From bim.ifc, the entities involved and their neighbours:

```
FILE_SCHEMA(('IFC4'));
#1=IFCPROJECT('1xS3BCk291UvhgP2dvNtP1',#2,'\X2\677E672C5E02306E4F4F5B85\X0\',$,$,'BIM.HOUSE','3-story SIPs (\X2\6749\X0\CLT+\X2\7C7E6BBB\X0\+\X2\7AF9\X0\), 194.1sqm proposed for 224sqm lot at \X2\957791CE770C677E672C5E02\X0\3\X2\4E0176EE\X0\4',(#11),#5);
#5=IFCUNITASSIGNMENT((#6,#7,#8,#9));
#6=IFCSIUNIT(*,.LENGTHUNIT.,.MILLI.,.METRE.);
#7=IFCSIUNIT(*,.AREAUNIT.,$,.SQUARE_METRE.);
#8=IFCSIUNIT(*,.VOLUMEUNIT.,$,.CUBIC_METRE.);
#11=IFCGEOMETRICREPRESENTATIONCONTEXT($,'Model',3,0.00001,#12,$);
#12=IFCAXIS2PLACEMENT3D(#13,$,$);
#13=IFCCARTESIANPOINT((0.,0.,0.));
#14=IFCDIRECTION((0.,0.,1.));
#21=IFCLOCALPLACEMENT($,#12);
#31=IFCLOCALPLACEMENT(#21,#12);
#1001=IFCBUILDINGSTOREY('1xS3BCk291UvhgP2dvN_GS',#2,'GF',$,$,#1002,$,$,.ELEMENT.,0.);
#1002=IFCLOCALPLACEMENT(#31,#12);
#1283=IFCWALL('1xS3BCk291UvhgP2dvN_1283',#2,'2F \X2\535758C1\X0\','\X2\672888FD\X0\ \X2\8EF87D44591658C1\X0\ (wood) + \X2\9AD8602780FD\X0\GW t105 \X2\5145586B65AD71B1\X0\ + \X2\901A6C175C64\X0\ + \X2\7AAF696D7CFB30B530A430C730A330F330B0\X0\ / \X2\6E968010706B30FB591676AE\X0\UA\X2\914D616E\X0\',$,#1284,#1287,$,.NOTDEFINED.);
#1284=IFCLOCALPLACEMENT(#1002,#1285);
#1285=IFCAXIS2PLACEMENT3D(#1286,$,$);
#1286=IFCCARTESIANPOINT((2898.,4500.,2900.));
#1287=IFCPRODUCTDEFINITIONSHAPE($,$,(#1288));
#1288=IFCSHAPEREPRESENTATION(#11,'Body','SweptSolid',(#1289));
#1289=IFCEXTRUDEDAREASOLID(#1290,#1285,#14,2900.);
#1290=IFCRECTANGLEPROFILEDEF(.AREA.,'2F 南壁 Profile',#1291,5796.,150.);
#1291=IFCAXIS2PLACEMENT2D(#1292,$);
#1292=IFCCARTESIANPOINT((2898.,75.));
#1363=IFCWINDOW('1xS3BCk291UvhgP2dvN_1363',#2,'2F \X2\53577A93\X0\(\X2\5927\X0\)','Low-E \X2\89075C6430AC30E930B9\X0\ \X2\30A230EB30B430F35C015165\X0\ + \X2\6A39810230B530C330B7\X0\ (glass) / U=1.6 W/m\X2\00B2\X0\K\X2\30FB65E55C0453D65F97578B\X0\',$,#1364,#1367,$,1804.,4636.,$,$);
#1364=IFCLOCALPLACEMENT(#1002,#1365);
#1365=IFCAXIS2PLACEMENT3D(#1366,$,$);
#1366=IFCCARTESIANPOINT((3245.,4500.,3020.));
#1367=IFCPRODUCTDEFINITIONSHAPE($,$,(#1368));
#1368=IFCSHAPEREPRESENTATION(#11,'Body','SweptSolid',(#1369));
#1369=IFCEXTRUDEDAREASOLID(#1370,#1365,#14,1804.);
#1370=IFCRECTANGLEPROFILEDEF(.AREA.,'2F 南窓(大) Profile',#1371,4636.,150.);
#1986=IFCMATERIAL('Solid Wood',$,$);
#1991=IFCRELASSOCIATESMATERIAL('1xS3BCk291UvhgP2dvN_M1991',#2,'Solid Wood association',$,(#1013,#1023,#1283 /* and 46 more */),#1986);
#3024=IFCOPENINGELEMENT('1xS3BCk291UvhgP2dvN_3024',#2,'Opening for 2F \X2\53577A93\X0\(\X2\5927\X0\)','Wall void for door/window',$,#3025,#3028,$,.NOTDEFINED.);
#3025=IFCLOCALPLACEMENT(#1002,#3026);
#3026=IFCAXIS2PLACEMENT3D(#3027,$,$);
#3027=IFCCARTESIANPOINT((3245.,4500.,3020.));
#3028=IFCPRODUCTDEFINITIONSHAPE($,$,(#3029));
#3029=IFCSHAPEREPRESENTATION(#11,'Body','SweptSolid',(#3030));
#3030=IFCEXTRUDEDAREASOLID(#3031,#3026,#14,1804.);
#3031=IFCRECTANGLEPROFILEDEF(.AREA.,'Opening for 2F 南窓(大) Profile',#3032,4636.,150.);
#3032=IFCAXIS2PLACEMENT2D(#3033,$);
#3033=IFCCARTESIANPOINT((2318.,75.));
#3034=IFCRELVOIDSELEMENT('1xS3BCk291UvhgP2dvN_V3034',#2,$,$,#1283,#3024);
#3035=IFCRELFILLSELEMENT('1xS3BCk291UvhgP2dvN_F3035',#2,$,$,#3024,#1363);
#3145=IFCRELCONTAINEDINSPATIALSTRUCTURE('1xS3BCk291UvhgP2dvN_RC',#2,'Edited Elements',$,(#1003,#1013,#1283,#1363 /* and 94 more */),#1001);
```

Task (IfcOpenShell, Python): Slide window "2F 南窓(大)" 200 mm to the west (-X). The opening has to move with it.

```python
import ifcopenshell
import ifcopenshell.api.geometry
import ifcopenshell.util.placement

model = ifcopenshell.open("bim.ifc")

window = model.by_guid("1xS3BCk291UvhgP2dvN_1363")
opening = window.FillsVoids[0].RelatingOpeningElement
wall = opening.VoidsElements[0].RelatingBuildingElement

wall_matrix = ifcopenshell.util.placement.get_local_placement(wall.ObjectPlacement)
shift = wall_matrix[:3, 0] * -200.0
before = ifcopenshell.util.placement.get_local_placement(window.ObjectPlacement)[:3, 3].copy()

# The window is not placed relative to its opening, so move both.
for product in (opening, window):
    matrix = ifcopenshell.util.placement.get_local_placement(product.ObjectPlacement)
    matrix[:3, 3] += shift
    ifcopenshell.api.geometry.edit_object_placement(model, product=product, matrix=matrix, is_si=False)

after = ifcopenshell.util.placement.get_local_placement(window.ObjectPlacement)[:3, 3]
print("window moved by", (after - before).round(3) + 0.0)

model.write("bim_v2.ifc")
```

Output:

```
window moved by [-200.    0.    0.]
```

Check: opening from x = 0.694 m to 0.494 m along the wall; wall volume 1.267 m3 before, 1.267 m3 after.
